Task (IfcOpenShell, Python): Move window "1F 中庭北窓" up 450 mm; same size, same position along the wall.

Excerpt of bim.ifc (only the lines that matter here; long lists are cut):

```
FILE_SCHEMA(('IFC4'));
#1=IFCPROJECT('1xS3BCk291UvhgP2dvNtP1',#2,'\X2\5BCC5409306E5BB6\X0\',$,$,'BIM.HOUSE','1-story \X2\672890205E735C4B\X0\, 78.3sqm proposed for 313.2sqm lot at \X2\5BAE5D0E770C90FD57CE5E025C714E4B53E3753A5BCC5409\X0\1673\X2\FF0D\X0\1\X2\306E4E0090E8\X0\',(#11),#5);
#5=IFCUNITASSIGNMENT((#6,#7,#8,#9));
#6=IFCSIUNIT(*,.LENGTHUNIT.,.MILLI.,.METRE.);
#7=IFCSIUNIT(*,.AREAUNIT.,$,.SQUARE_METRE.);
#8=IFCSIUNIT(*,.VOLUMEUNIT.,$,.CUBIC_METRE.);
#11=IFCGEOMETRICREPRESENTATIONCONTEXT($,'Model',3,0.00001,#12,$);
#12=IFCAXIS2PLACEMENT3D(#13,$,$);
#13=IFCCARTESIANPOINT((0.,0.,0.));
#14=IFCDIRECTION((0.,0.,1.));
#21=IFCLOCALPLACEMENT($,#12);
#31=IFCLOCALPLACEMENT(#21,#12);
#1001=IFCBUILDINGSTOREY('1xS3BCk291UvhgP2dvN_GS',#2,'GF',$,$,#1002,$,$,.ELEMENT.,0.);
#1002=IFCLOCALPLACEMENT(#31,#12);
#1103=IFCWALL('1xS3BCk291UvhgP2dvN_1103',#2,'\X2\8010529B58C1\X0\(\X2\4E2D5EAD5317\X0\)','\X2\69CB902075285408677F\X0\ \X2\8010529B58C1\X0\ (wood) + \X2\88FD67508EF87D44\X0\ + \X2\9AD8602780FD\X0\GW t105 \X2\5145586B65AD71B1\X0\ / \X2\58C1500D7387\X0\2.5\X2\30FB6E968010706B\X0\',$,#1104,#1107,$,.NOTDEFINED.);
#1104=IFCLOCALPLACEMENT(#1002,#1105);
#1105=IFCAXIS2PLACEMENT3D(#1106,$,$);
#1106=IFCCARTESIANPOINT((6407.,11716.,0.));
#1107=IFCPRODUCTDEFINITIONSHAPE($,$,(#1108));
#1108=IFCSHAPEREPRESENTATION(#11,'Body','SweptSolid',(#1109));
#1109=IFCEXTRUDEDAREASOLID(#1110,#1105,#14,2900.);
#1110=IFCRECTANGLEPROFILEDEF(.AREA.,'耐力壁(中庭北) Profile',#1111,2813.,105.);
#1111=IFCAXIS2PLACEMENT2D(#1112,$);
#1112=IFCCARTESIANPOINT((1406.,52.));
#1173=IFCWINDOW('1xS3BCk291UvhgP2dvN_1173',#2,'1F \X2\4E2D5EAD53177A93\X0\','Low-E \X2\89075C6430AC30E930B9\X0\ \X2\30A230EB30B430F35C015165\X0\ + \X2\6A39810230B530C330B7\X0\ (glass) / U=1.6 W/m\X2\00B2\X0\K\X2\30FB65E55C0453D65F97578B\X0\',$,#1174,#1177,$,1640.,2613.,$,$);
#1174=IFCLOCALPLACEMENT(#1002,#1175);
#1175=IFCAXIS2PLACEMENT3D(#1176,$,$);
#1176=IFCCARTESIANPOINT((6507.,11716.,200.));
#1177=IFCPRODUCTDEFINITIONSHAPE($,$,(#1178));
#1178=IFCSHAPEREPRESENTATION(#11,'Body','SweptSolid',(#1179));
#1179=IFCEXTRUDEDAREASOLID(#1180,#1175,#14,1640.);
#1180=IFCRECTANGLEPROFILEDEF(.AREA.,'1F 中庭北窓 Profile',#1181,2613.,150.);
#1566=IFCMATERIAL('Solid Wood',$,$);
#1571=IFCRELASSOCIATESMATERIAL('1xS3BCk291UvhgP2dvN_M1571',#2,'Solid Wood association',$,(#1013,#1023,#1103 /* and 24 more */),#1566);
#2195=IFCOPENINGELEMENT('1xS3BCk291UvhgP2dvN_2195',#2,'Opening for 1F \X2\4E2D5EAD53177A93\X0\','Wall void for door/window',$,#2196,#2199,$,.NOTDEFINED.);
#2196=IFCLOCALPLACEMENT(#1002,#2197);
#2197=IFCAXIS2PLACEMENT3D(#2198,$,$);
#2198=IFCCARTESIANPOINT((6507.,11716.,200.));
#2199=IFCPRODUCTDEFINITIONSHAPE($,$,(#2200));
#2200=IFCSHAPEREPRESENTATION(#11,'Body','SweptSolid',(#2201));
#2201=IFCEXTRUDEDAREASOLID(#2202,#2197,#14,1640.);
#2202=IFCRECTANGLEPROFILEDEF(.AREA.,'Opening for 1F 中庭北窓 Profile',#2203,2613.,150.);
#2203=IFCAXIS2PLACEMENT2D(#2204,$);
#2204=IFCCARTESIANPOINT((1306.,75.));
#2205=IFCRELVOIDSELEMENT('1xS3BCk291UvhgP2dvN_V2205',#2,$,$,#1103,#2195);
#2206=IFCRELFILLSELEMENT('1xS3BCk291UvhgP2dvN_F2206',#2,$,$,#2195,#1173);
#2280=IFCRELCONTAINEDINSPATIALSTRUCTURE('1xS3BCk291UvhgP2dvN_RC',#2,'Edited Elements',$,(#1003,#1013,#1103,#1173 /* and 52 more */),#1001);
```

```python
import numpy as np
import ifcopenshell
import ifcopenshell.api.geometry
import ifcopenshell.util.placement
import ifcopenshell.util.unit

model = ifcopenshell.open("bim.ifc")
unit_scale = ifcopenshell.util.unit.calculate_unit_scale(model)

window = model.by_id(1173)
opening = window.FillsVoids[0].RelatingOpeningElement
dz = 0.45 / unit_scale

shift = np.array([0.0, 0.0, dz])
# The window is not placed relative to its opening, so move both.
for product in (opening, window):
    matrix = ifcopenshell.util.placement.get_local_placement(product.ObjectPlacement)
    matrix[:3, 3] += shift
    ifcopenshell.api.geometry.edit_object_placement(model, product=product, matrix=matrix, is_si=False)

print(f"moved by {dz * unit_scale:+.3f} m")

model.write("bim-out.ifc")
```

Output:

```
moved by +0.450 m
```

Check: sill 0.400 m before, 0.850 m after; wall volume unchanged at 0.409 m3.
